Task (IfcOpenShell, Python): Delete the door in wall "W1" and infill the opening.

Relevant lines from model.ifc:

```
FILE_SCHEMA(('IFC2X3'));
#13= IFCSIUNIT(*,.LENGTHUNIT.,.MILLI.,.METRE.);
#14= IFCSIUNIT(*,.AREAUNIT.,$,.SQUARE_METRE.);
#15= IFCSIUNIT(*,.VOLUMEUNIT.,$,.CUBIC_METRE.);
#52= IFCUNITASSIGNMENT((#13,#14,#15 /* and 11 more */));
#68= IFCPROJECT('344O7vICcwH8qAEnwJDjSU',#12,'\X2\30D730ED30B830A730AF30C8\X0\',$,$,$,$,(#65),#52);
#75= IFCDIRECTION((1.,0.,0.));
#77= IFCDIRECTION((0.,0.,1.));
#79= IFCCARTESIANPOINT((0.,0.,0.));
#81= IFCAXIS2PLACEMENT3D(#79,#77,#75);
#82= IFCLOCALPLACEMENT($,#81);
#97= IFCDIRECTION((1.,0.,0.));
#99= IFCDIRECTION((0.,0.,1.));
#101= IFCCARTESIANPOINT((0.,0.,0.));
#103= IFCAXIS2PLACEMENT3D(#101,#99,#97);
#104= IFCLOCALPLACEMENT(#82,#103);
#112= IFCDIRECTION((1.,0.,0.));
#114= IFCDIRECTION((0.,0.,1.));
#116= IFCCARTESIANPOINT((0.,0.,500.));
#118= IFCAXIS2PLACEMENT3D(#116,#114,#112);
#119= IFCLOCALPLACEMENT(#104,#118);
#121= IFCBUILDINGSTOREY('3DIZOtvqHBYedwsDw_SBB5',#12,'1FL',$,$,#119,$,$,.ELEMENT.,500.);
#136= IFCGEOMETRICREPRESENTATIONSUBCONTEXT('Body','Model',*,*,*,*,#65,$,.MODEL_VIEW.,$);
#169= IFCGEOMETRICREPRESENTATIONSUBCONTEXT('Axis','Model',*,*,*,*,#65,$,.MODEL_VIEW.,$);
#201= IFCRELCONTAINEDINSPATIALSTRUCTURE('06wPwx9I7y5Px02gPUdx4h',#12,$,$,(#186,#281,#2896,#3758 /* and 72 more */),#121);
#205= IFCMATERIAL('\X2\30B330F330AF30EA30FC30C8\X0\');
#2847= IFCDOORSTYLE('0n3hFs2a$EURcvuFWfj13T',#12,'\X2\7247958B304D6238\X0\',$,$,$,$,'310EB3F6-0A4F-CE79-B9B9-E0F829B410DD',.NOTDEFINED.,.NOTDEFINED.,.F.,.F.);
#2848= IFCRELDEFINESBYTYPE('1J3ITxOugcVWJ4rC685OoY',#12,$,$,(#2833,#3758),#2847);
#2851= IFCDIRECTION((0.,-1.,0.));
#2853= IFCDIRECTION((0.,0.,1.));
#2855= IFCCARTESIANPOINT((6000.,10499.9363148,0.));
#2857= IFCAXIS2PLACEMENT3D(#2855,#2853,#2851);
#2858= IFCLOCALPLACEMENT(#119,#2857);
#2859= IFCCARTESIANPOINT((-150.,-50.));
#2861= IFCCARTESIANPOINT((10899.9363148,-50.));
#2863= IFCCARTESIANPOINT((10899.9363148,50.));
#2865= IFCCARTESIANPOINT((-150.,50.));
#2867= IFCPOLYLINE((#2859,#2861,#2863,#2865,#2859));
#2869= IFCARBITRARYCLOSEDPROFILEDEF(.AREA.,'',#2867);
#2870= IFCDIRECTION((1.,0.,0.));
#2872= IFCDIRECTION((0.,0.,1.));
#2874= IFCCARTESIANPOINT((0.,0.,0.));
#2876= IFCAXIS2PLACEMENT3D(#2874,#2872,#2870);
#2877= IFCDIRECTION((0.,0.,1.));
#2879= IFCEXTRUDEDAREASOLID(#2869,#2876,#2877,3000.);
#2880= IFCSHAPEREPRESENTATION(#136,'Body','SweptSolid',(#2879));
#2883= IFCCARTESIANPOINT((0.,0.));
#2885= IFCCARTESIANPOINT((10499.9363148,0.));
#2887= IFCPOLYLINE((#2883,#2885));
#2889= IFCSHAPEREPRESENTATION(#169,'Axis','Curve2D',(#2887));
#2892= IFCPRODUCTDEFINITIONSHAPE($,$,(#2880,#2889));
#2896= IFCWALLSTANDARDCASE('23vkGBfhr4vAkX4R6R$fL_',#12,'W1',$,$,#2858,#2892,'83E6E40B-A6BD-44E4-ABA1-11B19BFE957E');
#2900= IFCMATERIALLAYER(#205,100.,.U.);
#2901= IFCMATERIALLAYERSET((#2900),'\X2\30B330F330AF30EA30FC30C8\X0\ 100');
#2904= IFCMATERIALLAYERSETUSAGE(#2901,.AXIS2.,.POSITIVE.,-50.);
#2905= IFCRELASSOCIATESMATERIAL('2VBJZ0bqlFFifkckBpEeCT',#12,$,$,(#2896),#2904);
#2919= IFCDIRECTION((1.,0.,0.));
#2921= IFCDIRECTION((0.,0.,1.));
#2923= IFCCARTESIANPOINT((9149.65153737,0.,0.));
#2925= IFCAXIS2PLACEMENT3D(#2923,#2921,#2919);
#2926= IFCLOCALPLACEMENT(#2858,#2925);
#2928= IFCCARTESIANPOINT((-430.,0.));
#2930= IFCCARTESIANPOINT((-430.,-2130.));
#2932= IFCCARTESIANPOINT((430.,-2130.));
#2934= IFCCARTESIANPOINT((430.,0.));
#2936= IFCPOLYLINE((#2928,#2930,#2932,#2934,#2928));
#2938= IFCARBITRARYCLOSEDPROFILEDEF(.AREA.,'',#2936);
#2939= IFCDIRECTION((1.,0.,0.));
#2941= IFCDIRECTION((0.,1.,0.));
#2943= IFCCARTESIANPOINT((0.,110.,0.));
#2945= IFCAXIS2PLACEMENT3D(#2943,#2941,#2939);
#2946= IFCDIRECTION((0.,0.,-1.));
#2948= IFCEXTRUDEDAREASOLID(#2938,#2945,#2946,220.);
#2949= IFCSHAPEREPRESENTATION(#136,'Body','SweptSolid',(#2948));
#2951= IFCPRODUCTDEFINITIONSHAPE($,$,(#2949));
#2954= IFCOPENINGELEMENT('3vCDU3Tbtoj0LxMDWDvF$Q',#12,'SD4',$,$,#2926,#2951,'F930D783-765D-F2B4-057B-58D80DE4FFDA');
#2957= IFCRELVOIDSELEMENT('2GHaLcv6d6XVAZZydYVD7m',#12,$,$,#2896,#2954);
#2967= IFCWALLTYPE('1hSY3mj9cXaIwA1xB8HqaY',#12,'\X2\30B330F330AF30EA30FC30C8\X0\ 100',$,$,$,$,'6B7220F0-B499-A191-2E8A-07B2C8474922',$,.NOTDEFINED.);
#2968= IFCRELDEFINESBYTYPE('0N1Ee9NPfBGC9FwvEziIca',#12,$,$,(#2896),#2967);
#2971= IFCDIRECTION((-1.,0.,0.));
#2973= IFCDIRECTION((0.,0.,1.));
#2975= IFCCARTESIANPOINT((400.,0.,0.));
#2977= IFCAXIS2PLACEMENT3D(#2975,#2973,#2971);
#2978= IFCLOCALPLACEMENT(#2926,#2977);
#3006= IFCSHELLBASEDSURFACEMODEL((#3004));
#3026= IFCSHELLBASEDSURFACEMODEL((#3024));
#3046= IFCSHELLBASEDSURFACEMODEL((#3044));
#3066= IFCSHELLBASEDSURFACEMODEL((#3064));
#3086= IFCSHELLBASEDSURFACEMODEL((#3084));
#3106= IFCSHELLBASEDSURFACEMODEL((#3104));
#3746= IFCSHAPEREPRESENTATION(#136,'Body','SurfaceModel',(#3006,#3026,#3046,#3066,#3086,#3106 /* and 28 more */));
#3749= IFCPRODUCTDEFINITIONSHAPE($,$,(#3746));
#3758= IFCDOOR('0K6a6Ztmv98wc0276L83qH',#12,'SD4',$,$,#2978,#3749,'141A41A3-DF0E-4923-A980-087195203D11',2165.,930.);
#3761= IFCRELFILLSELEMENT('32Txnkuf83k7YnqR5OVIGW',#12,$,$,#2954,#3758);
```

```python
import ifcopenshell
import ifcopenshell.api.feature
import ifcopenshell.api.root
import ifcopenshell.geom
import ifcopenshell.util.shape

model = ifcopenshell.open("model.ifc")
settings = ifcopenshell.geom.settings()


def volume(element):
    """Net volume in cubic metres, openings subtracted."""
    shape = ifcopenshell.geom.create_shape(settings, element)
    return ifcopenshell.util.shape.get_volume(shape.geometry)


door = model.by_guid("0K6a6Ztmv98wc0276L83qH")
opening = door.FillsVoids[0].RelatingOpeningElement
wall = opening.VoidsElements[0].RelatingBuildingElement
before = volume(wall)

ifcopenshell.api.root.remove_product(model, product=door)
ifcopenshell.api.feature.remove_feature(model, feature=opening)

after = volume(wall)

print(f"wall volume {before:.3f} -> {after:.3f} m3")

model.write("model-out.ifc")
```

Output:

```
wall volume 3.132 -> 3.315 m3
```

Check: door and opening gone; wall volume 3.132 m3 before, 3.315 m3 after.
